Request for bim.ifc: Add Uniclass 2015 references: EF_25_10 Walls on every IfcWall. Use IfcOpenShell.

First a look at what the model holds.

```python
import ifcopenshell

model = ifcopenshell.open("bim.ifc")
print(model.schema)
print("classifications:", [c.Name for c in model.by_type("IfcClassification")])
for ifc_class in ("IfcDoor", "IfcRoof", "IfcStair", "IfcWall", "IfcWindow"):
    print(ifc_class, len(model.by_type(ifc_class)))
```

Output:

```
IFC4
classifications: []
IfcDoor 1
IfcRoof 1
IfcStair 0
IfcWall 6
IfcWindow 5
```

```python
import ifcopenshell
import ifcopenshell.api.classification

model = ifcopenshell.open("bim.ifc")

system = ifcopenshell.api.classification.add_classification(model, classification="Uniclass 2015")

codes = {
    "IfcWall": ("EF_25_10", "Walls"),
}
for ifc_class, (code, name) in codes.items():
    products = model.by_type(ifc_class)
    ifcopenshell.api.classification.add_reference(
        model, products=products, classification=system, identification=code, name=name
    )
    print(code, len(products))

model.write("bim_rev.ifc")
```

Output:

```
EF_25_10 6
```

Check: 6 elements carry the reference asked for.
